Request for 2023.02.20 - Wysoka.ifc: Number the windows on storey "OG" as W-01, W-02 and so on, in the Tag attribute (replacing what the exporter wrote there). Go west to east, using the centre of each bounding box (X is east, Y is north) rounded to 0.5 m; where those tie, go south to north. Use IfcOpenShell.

First a look at what the model holds.

```python
import ifcopenshell
import ifcopenshell.util.element
import ifcopenshell.util.placement

model = ifcopenshell.open("2023.02.20 - Wysoka.ifc")
print(model.schema)
storey = next(s for s in model.by_type("IfcBuildingStorey") if s.Name == "OG")
windows = [e for e in ifcopenshell.util.element.get_decomposition(storey) if e.is_a("IfcWindow")]
for e in sorted(windows, key=lambda e: e.id()):
    origin = ifcopenshell.util.placement.get_local_placement(e.ObjectPlacement)[:3, 3]
    print(e.id(), e.Tag, e.Name, origin.round(2) + 0.0, sep=" | ")
```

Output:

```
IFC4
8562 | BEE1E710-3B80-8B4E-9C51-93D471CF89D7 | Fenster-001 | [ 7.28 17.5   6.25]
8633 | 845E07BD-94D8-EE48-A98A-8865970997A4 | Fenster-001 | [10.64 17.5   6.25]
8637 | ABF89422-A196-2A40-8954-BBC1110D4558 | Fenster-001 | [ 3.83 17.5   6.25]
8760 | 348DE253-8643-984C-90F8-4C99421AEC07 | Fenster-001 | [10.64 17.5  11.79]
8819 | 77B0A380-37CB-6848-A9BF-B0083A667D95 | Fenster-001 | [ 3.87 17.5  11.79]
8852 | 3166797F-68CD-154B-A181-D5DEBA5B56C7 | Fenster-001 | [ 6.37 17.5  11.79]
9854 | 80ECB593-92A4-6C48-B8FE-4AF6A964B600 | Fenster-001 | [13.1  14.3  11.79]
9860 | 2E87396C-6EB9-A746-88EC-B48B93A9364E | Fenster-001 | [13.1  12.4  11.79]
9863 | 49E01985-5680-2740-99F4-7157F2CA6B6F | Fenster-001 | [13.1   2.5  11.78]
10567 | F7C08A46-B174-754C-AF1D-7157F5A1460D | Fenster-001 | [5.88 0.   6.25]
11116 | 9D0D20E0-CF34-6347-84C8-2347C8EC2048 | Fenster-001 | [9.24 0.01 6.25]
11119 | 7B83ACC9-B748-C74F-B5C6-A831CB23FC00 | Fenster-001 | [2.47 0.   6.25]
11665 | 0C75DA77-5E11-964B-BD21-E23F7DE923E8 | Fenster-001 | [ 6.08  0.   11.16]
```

```python
import ifcopenshell
import ifcopenshell.geom
import ifcopenshell.util.element
import ifcopenshell.util.shape

model = ifcopenshell.open("2023.02.20 - Wysoka.ifc")
settings = ifcopenshell.geom.settings()
settings.set("use-world-coords", True)


def centre(element):
    shape = ifcopenshell.geom.create_shape(settings, element)
    return ifcopenshell.util.shape.get_bbox_centroid(shape.geometry)


storey = next(s for s in model.by_type("IfcBuildingStorey") if s.Name == "OG")
windows = [e for e in ifcopenshell.util.element.get_decomposition(storey) if e.is_a("IfcWindow")]

# Insertion points can sit at a corner or the storey origin, so sort by the geometry (in metres).
centres = {e: centre(e) for e in windows}
windows.sort(key=lambda e: (round(centres[e][0] / 0.5), centres[e][1]))

for i, e in enumerate(windows, start=1):
    number = f"W-{i:02d}"
    e.Tag = number
    print(e.id(), number)

model.write("2023.02.20 - Wysoka_rev.ifc")
```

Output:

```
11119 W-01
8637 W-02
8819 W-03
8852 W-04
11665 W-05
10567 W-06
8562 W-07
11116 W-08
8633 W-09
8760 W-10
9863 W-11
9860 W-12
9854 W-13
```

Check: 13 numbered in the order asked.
